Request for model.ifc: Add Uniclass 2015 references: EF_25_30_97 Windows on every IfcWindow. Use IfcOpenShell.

First a look at what the model holds.

```python
import ifcopenshell

model = ifcopenshell.open("model.ifc")
print(model.schema)
print("classifications:", [c.Name for c in model.by_type("IfcClassification")])
for ifc_class in ("IfcDoor", "IfcRoof", "IfcStair", "IfcWall", "IfcWindow"):
    print(ifc_class, len(model.by_type(ifc_class)))
```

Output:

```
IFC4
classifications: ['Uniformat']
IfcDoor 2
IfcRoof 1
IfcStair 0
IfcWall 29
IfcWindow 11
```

```python
import ifcopenshell
import ifcopenshell.api.classification

model = ifcopenshell.open("model.ifc")

system = ifcopenshell.api.classification.add_classification(model, classification="Uniclass 2015")

codes = {
    "IfcWindow": ("EF_25_30_97", "Windows"),
}
for ifc_class, (code, name) in codes.items():
    products = model.by_type(ifc_class)
    ifcopenshell.api.classification.add_reference(
        model, products=products, classification=system, identification=code, name=name
    )
    print(code, len(products))

model.write("model_v2.ifc")
```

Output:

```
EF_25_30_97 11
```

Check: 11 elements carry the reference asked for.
